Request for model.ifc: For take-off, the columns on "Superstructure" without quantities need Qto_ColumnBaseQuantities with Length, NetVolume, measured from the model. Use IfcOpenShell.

First a look at what the model holds.

```python
import ifcopenshell
import ifcopenshell.util.element
import ifcopenshell.util.unit

model = ifcopenshell.open("model.ifc")
print(model.schema)
for unit_type in ("LENGTHUNIT", "AREAUNIT", "VOLUMEUNIT"):
    print(unit_type, ifcopenshell.util.unit.calculate_unit_scale(model, unit_type))
storey = next(s for s in model.by_type("IfcBuildingStorey") if s.Name == "Superstructure")
columns = [e for e in ifcopenshell.util.element.get_decomposition(storey) if e.is_a("IfcColumn")]
for e in sorted(columns, key=lambda e: e.id()):
    print(e.id(), e.is_a(), e.Name, list(ifcopenshell.util.element.get_psets(e, qtos_only=True)), sep=" | ")
```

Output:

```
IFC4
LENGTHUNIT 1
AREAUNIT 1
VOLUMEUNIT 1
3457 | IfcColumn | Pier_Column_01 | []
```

```python
import ifcopenshell
import ifcopenshell.api.pset
import ifcopenshell.geom
import ifcopenshell.util.element
import ifcopenshell.util.shape
import ifcopenshell.util.unit

model = ifcopenshell.open("model.ifc")
unit_scale = ifcopenshell.util.unit.calculate_unit_scale(model)
volume_scale = ifcopenshell.util.unit.calculate_unit_scale(model, "VOLUMEUNIT")
settings = ifcopenshell.geom.settings()

storey = next(s for s in model.by_type("IfcBuildingStorey") if s.Name == "Superstructure")
columns = [e for e in ifcopenshell.util.element.get_decomposition(storey) if e.is_a("IfcColumn")]

for e in sorted(columns, key=lambda e: e.id()):
    if ifcopenshell.util.element.get_psets(e, qtos_only=True, should_inherit=False):
        continue
    # Geometry comes back in metres, in the element's own axes.
    shape = ifcopenshell.geom.create_shape(settings, e)
    values = {
        "Length": ifcopenshell.util.shape.get_z(shape.geometry) / unit_scale,
        "NetVolume": ifcopenshell.util.shape.get_volume(shape.geometry) / volume_scale,
    }
    qto = ifcopenshell.api.pset.add_qto(model, product=e, name="Qto_ColumnBaseQuantities")
    ifcopenshell.api.pset.edit_qto(model, qto=qto, properties=values)
    print(e.id(), {k: round(v, 3) for k, v in values.items()})

model.write("model_v2.ifc")
```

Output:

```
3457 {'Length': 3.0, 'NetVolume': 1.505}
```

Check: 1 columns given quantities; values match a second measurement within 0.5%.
